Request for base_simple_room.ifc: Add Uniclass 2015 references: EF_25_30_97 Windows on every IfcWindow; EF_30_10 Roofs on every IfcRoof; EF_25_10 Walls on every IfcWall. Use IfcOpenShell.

First a look at what the model holds.

```python
import ifcopenshell

model = ifcopenshell.open("base_simple_room.ifc")
print(model.schema)
print("classifications:", [c.Name for c in model.by_type("IfcClassification")])
for ifc_class in ("IfcDoor", "IfcRoof", "IfcStair", "IfcWall", "IfcWindow"):
    print(ifc_class, len(model.by_type(ifc_class)))
```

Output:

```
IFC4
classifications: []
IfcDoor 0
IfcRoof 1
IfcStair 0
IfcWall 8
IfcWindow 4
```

```python
import ifcopenshell
import ifcopenshell.api.classification

model = ifcopenshell.open("base_simple_room.ifc")

system = ifcopenshell.api.classification.add_classification(model, classification="Uniclass 2015")

codes = {
    "IfcWindow": ("EF_25_30_97", "Windows"),
    "IfcRoof": ("EF_30_10", "Roofs"),
    "IfcWall": ("EF_25_10", "Walls"),
}
for ifc_class, (code, name) in codes.items():
    products = model.by_type(ifc_class)
    ifcopenshell.api.classification.add_reference(
        model, products=products, classification=system, identification=code, name=name
    )
    print(code, len(products))

model.write("base_simple_room_edited.ifc")
```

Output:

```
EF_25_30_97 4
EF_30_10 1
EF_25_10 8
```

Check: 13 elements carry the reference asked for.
